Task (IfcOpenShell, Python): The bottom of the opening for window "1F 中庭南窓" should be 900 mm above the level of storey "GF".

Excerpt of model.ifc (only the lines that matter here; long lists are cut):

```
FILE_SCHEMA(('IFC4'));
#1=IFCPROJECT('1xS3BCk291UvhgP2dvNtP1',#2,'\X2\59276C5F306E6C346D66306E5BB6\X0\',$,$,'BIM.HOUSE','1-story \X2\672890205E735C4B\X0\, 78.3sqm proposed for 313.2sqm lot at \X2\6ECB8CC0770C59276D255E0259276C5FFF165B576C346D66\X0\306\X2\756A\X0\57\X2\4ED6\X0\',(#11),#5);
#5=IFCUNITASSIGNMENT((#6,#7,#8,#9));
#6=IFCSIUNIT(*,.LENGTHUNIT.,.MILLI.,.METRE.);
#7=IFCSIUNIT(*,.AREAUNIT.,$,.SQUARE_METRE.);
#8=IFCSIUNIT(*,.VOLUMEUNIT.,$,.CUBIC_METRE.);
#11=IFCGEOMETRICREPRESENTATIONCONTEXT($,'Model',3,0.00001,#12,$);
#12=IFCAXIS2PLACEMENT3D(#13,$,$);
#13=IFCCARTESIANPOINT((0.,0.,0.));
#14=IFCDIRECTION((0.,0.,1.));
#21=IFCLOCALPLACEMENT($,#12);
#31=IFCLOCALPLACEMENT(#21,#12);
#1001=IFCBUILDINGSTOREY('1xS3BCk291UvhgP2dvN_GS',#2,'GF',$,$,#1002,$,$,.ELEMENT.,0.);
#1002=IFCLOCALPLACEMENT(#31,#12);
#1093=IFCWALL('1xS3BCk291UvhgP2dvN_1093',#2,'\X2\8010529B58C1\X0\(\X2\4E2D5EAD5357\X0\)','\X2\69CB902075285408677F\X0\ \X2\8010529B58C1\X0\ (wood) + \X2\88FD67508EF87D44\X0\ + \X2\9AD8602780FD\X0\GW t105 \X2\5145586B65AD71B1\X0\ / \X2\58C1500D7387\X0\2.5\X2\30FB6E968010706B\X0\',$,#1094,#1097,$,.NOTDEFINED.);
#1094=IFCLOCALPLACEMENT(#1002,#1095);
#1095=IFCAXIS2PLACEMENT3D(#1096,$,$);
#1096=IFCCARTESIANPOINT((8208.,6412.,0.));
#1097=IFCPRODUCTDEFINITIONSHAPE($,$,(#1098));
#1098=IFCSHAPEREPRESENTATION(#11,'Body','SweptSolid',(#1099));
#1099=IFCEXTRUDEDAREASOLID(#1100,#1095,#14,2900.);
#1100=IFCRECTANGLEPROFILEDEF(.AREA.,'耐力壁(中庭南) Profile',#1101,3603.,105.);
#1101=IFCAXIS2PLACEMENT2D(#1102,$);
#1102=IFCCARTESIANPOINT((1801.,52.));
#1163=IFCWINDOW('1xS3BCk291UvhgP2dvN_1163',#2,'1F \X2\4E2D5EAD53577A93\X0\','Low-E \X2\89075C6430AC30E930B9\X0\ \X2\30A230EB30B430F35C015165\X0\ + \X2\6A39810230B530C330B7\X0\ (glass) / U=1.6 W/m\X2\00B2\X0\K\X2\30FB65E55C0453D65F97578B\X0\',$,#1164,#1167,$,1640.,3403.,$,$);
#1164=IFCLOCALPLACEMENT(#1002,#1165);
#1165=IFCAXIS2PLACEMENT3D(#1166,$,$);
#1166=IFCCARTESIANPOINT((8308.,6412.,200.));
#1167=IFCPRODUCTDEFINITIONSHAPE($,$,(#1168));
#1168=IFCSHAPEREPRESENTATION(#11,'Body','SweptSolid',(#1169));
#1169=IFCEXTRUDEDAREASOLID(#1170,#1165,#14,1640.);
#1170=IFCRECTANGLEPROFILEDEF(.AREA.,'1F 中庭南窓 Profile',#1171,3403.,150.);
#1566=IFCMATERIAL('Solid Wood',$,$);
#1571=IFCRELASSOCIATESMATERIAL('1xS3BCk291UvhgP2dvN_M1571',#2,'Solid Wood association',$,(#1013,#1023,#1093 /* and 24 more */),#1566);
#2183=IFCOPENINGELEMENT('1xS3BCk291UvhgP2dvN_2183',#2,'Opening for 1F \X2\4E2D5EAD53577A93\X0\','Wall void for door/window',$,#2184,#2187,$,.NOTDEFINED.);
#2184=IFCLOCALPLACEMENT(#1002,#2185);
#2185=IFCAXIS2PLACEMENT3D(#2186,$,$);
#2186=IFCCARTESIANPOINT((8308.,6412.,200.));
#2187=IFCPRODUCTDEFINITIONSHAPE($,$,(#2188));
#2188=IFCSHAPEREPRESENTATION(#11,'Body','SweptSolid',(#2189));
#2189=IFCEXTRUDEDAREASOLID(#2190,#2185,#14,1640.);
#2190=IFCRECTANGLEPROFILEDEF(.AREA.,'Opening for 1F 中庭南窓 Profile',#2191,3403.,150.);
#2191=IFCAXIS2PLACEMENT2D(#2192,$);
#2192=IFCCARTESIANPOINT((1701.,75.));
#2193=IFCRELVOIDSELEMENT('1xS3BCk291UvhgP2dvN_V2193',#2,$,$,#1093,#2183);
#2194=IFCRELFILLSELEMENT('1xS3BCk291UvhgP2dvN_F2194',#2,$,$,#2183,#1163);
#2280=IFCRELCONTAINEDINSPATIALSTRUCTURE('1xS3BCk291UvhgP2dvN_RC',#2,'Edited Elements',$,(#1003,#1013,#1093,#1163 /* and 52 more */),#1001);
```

```python
import numpy as np
import ifcopenshell
import ifcopenshell.api.geometry
import ifcopenshell.geom
import ifcopenshell.util.element
import ifcopenshell.util.placement
import ifcopenshell.util.shape
import ifcopenshell.util.unit

model = ifcopenshell.open("model.ifc")
unit_scale = ifcopenshell.util.unit.calculate_unit_scale(model)

window = model.by_id(1163)
opening = window.FillsVoids[0].RelatingOpeningElement
storey = ifcopenshell.util.element.get_container(window, ifc_class="IfcBuildingStorey")
level = ifcopenshell.util.placement.get_local_placement(storey.ObjectPlacement)[2, 3]

# The opening's origin need not be at the sill, so measure its lowest point.
shape = ifcopenshell.geom.create_shape(ifcopenshell.geom.settings(), opening)
bottom = ifcopenshell.util.shape.get_shape_bottom_elevation(shape, shape.geometry) / unit_scale
dz = level + 900.0 - bottom

shift = np.array([0.0, 0.0, dz])
# The window is not placed relative to its opening, so move both.
for product in (opening, window):
    matrix = ifcopenshell.util.placement.get_local_placement(product.ObjectPlacement)
    matrix[:3, 3] += shift
    ifcopenshell.api.geometry.edit_object_placement(model, product=product, matrix=matrix, is_si=False)

print(f"moved by {dz * unit_scale:+.3f} m")

model.write("model_edited.ifc")
```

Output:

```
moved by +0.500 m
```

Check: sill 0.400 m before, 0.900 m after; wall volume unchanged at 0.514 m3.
